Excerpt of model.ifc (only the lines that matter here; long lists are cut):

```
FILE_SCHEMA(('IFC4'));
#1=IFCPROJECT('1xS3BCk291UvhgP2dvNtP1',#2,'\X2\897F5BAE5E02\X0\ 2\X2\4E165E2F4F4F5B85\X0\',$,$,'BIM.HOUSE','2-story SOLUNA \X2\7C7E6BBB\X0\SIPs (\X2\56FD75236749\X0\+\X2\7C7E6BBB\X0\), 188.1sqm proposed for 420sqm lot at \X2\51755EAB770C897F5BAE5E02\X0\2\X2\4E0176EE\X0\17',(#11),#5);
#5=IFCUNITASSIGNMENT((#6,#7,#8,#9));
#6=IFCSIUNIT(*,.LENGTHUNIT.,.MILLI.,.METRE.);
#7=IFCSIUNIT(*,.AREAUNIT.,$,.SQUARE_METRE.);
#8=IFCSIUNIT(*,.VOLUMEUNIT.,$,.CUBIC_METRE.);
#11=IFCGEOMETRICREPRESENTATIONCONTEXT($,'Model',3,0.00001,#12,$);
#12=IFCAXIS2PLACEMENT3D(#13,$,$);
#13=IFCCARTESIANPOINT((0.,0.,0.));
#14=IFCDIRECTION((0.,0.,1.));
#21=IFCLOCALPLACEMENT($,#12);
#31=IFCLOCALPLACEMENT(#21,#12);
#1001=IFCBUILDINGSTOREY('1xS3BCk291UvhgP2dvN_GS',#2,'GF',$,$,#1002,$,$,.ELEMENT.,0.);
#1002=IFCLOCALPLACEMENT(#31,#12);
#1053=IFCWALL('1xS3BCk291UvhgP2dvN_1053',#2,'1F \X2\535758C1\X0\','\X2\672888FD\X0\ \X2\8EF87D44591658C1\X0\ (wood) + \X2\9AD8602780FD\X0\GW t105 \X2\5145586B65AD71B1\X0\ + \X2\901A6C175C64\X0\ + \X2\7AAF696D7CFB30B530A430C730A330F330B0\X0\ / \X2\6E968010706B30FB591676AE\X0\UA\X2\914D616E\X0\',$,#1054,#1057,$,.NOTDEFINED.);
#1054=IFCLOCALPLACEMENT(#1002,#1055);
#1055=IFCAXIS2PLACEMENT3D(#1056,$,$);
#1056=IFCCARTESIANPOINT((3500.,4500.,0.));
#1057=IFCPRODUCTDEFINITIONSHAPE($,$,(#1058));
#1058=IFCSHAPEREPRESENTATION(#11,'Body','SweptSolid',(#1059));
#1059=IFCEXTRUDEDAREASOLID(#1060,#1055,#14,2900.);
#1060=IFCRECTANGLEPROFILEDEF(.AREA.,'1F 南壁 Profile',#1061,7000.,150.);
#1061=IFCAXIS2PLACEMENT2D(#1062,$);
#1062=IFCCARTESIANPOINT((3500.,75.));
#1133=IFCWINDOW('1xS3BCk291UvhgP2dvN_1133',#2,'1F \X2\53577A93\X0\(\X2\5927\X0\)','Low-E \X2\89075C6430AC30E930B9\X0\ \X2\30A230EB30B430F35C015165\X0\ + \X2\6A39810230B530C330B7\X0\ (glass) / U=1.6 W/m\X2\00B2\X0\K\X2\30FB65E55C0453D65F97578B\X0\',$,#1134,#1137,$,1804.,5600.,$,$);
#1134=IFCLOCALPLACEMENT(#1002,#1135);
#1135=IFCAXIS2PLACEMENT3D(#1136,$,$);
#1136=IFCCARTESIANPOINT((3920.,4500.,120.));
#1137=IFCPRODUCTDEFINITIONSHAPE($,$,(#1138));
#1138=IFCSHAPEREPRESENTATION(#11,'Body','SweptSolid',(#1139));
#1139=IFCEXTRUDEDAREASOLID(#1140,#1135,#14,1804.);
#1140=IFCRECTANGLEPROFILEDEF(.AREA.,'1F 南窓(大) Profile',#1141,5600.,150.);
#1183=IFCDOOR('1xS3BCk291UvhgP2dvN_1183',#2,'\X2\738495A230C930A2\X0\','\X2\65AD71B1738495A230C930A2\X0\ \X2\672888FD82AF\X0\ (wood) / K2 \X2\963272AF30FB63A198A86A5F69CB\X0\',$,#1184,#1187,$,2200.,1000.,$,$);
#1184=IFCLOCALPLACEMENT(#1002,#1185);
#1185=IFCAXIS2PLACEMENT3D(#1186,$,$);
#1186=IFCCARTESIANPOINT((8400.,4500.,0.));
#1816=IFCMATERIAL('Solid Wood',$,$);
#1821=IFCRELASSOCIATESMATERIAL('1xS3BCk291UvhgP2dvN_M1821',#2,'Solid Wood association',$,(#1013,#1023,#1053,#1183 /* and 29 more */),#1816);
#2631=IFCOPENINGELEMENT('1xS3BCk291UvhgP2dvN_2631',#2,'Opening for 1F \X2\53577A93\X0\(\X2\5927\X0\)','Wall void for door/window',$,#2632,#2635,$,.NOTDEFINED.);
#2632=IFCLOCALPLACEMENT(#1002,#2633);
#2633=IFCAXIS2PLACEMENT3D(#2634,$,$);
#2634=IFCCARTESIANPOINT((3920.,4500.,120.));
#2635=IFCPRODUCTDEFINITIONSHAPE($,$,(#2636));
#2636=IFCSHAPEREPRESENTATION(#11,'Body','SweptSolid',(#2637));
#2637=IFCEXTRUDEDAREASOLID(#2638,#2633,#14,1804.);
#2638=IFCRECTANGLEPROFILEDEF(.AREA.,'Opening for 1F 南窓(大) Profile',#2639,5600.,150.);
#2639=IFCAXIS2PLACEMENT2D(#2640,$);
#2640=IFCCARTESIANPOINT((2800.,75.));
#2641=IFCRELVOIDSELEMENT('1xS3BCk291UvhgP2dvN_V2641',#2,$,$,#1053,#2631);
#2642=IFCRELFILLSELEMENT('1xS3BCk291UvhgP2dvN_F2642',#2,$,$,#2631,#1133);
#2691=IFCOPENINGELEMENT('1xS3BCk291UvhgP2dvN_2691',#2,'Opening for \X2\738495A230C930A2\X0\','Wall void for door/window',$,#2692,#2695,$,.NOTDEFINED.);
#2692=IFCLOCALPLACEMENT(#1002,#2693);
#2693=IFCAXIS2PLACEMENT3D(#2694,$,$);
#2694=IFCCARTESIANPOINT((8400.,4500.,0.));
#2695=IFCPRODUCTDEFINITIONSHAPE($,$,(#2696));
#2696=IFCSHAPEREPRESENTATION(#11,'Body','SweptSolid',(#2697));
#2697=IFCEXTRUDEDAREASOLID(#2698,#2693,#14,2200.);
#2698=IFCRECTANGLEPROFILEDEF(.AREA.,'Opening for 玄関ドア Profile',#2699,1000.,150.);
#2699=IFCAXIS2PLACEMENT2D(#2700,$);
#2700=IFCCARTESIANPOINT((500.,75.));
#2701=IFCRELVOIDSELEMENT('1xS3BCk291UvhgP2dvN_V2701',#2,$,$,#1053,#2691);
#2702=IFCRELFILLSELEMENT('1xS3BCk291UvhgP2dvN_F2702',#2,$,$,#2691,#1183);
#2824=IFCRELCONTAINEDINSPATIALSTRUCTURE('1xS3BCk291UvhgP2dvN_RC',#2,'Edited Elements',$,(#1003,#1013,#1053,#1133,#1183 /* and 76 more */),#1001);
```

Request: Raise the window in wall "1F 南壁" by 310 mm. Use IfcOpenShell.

```python
import numpy as np
import ifcopenshell
import ifcopenshell.api.geometry
import ifcopenshell.util.placement
import ifcopenshell.util.unit

model = ifcopenshell.open("model.ifc")
unit_scale = ifcopenshell.util.unit.calculate_unit_scale(model)

window = model.by_guid("1xS3BCk291UvhgP2dvN_1133")
opening = window.FillsVoids[0].RelatingOpeningElement
dz = 0.31 / unit_scale

shift = np.array([0.0, 0.0, dz])
# The window is not placed relative to its opening, so move both.
for product in (opening, window):
    matrix = ifcopenshell.util.placement.get_local_placement(product.ObjectPlacement)
    matrix[:3, 3] += shift
    ifcopenshell.api.geometry.edit_object_placement(model, product=product, matrix=matrix, is_si=False)

print(f"moved by {dz * unit_scale:+.3f} m")

model.write("model_v2.ifc")
```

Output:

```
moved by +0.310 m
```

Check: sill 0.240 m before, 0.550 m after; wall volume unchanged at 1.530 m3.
